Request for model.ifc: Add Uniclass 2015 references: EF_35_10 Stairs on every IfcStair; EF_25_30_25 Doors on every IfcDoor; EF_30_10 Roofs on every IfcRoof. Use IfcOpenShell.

First a look at what the model holds.

```python
import ifcopenshell

model = ifcopenshell.open("model.ifc")
print(model.schema)
print("classifications:", [c.Name for c in model.by_type("IfcClassification")])
for ifc_class in ("IfcDoor", "IfcRoof", "IfcStair", "IfcWall", "IfcWindow"):
    print(ifc_class, len(model.by_type(ifc_class)))
```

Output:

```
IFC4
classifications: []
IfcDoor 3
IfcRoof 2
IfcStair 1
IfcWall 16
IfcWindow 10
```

```python
import ifcopenshell
import ifcopenshell.api.classification

model = ifcopenshell.open("model.ifc")

system = ifcopenshell.api.classification.add_classification(model, classification="Uniclass 2015")

codes = {
    "IfcStair": ("EF_35_10", "Stairs"),
    "IfcDoor": ("EF_25_30_25", "Doors"),
    "IfcRoof": ("EF_30_10", "Roofs"),
}
for ifc_class, (code, name) in codes.items():
    products = model.by_type(ifc_class)
    ifcopenshell.api.classification.add_reference(
        model, products=products, classification=system, identification=code, name=name
    )
    print(code, len(products))

model.write("model_rev.ifc")
```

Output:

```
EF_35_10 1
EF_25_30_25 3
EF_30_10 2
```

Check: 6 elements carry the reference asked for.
